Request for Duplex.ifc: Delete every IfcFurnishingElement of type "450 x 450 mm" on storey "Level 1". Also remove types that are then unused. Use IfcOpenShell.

First a look at what the model holds.

```python
import ifcopenshell
import ifcopenshell.util.element

model = ifcopenshell.open("Duplex.ifc")
print(model.schema)
storey = next(s for s in model.by_type("IfcBuildingStorey") if s.Name == "Level 1")
furniture = [e for e in ifcopenshell.util.element.get_decomposition(storey) if e.is_a("IfcFurnishingElement")]
seen = {}
for e in furniture:
    element_type = ifcopenshell.util.element.get_type(e)
    name = element_type.Name if element_type not in (None, e) else None
    seen[name] = seen.get(name, 0) + 1
for name, count in sorted(seen.items(), key=str):
    print(count, "x", name)
```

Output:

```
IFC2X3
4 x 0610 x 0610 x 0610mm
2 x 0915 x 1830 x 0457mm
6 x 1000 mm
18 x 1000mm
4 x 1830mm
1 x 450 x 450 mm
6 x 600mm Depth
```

```python
import ifcopenshell
import ifcopenshell.api.root
import ifcopenshell.util.element

model = ifcopenshell.open("Duplex.ifc")

storey = next(s for s in model.by_type("IfcBuildingStorey") if s.Name == "Level 1")
furniture = [e for e in ifcopenshell.util.element.get_decomposition(storey) if e.is_a("IfcFurnishingElement")]
targets = [e for e in furniture if (t := ifcopenshell.util.element.get_type(e)) not in (None, e) and t.Name == "450 x 450 mm"]
types = {ifcopenshell.util.element.get_type(e) for e in targets} - {None, *targets}

for e in targets:
    ifcopenshell.api.root.remove_product(model, product=e)
print(len(targets), "removed")

unused = [t for t in types if not ifcopenshell.util.element.get_types(t)]
for t in unused:
    ifcopenshell.api.root.remove_product(model, product=t)
print(len(unused), "unused types removed")

model.write("Duplex-out.ifc")
```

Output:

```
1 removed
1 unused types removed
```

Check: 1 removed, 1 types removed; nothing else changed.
